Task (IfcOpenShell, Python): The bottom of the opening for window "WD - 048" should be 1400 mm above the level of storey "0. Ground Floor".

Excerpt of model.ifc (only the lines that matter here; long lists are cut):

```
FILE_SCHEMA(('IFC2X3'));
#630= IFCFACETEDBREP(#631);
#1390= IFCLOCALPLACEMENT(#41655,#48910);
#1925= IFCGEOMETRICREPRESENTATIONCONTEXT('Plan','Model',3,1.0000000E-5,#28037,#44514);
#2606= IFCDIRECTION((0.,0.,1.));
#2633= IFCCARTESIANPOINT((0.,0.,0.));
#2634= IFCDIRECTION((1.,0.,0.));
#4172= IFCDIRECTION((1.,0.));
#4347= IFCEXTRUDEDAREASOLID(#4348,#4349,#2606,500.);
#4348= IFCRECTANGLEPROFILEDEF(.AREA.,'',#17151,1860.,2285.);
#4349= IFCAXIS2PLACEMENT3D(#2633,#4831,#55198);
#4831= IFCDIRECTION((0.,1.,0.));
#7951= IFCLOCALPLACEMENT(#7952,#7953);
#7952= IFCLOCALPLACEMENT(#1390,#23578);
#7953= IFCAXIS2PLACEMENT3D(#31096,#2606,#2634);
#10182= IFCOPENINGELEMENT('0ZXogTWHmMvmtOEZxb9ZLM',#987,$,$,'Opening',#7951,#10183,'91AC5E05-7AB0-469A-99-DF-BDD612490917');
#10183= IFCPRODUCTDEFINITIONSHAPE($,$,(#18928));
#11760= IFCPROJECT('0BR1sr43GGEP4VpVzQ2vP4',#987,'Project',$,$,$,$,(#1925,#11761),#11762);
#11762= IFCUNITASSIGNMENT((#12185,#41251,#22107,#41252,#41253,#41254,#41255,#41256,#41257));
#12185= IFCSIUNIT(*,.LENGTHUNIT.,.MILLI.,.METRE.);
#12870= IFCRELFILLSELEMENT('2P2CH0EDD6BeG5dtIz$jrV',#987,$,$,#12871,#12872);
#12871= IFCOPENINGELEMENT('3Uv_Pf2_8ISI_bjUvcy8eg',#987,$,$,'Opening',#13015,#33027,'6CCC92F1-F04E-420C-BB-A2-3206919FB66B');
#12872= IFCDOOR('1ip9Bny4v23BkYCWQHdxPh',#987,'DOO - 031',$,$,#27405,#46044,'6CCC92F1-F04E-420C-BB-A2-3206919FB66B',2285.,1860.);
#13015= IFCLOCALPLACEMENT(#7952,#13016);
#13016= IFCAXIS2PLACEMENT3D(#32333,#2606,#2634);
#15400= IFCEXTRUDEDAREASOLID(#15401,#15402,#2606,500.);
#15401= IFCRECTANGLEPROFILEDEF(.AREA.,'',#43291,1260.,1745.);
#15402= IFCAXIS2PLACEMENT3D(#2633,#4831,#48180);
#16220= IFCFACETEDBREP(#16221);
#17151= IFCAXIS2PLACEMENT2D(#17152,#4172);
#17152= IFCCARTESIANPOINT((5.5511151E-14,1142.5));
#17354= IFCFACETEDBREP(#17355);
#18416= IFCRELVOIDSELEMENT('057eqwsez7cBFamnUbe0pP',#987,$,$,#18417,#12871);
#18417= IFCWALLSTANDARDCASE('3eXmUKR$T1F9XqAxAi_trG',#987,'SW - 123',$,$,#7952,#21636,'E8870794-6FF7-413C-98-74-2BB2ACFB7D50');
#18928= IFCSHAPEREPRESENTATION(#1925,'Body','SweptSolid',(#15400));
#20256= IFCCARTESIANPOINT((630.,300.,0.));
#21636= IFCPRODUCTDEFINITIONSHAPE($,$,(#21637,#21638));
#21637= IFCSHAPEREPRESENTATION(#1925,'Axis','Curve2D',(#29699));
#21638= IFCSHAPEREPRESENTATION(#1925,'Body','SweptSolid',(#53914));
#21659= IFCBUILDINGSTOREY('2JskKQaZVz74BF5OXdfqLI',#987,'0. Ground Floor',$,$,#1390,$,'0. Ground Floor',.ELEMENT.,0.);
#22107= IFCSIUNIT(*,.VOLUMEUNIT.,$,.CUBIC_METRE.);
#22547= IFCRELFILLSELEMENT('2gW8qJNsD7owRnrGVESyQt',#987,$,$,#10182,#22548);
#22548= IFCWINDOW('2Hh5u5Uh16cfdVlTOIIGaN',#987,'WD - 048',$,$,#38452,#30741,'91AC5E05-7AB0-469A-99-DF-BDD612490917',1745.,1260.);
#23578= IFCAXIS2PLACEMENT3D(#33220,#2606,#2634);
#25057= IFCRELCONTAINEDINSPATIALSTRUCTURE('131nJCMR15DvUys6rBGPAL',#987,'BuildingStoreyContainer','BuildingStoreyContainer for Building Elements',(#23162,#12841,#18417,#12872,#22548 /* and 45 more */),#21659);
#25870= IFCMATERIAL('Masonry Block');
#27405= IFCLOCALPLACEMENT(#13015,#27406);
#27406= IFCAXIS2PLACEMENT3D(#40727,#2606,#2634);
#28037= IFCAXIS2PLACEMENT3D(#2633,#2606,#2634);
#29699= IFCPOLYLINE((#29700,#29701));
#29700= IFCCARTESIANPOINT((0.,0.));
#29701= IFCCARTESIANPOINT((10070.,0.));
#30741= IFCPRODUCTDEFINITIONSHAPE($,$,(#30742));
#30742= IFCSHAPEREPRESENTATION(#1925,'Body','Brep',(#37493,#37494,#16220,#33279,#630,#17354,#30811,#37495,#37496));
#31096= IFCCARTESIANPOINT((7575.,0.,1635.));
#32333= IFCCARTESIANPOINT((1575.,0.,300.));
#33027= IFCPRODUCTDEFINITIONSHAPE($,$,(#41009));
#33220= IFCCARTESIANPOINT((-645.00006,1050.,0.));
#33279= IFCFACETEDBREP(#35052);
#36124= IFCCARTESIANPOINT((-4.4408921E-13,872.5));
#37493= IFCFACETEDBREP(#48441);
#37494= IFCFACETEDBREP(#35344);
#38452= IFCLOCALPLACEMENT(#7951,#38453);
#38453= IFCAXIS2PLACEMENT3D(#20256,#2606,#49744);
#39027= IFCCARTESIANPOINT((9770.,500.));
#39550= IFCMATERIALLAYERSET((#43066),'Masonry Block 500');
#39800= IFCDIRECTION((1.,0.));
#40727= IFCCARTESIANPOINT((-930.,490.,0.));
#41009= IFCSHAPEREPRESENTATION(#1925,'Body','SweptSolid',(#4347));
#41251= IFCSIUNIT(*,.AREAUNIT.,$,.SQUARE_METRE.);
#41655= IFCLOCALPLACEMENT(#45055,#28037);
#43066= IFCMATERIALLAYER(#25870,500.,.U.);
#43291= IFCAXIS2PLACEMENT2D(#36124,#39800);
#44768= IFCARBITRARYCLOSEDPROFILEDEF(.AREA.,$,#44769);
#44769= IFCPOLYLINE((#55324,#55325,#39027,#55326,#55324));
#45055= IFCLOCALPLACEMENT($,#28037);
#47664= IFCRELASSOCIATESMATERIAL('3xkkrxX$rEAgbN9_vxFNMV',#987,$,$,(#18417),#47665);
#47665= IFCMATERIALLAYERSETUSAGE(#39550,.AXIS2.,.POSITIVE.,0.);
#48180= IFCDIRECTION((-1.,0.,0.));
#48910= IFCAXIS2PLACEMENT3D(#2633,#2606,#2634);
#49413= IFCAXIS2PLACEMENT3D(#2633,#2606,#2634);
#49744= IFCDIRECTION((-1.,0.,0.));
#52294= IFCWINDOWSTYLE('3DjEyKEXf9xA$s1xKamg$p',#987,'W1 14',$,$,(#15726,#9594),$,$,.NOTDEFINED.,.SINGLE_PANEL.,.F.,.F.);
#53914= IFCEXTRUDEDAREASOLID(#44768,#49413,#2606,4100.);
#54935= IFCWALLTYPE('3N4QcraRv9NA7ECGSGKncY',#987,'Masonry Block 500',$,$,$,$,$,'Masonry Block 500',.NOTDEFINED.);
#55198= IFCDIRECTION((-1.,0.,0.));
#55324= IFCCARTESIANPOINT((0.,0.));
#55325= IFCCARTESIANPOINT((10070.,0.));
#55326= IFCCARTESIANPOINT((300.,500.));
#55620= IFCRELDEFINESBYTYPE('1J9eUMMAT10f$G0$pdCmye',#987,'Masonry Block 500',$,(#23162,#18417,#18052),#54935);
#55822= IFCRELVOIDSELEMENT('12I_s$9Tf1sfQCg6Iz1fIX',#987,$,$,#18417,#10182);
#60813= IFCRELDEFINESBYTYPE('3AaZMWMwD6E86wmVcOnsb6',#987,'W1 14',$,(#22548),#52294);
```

```python
import numpy as np
import ifcopenshell
import ifcopenshell.api.geometry
import ifcopenshell.geom
import ifcopenshell.util.element
import ifcopenshell.util.placement
import ifcopenshell.util.shape
import ifcopenshell.util.unit

model = ifcopenshell.open("model.ifc")
unit_scale = ifcopenshell.util.unit.calculate_unit_scale(model)

window = model.by_guid("2Hh5u5Uh16cfdVlTOIIGaN")
opening = window.FillsVoids[0].RelatingOpeningElement
storey = ifcopenshell.util.element.get_container(window, ifc_class="IfcBuildingStorey")
level = ifcopenshell.util.placement.get_local_placement(storey.ObjectPlacement)[2, 3]

# The opening's origin need not be at the sill, so measure its lowest point.
shape = ifcopenshell.geom.create_shape(ifcopenshell.geom.settings(), opening)
bottom = ifcopenshell.util.shape.get_shape_bottom_elevation(shape, shape.geometry) / unit_scale
dz = level + 1400.0 - bottom

shift = np.array([0.0, 0.0, dz])
# The window is placed relative to its opening, so it follows when the opening moves.
matrix = ifcopenshell.util.placement.get_local_placement(opening.ObjectPlacement)
matrix[:3, 3] += shift
ifcopenshell.api.geometry.edit_object_placement(
    model, product=opening, matrix=matrix, is_si=False, should_transform_children=True
)

print(f"moved by {dz * unit_scale:+.3f} m")

model.write("model_rev.ifc")
```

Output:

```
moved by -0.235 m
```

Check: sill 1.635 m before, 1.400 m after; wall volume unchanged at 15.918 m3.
